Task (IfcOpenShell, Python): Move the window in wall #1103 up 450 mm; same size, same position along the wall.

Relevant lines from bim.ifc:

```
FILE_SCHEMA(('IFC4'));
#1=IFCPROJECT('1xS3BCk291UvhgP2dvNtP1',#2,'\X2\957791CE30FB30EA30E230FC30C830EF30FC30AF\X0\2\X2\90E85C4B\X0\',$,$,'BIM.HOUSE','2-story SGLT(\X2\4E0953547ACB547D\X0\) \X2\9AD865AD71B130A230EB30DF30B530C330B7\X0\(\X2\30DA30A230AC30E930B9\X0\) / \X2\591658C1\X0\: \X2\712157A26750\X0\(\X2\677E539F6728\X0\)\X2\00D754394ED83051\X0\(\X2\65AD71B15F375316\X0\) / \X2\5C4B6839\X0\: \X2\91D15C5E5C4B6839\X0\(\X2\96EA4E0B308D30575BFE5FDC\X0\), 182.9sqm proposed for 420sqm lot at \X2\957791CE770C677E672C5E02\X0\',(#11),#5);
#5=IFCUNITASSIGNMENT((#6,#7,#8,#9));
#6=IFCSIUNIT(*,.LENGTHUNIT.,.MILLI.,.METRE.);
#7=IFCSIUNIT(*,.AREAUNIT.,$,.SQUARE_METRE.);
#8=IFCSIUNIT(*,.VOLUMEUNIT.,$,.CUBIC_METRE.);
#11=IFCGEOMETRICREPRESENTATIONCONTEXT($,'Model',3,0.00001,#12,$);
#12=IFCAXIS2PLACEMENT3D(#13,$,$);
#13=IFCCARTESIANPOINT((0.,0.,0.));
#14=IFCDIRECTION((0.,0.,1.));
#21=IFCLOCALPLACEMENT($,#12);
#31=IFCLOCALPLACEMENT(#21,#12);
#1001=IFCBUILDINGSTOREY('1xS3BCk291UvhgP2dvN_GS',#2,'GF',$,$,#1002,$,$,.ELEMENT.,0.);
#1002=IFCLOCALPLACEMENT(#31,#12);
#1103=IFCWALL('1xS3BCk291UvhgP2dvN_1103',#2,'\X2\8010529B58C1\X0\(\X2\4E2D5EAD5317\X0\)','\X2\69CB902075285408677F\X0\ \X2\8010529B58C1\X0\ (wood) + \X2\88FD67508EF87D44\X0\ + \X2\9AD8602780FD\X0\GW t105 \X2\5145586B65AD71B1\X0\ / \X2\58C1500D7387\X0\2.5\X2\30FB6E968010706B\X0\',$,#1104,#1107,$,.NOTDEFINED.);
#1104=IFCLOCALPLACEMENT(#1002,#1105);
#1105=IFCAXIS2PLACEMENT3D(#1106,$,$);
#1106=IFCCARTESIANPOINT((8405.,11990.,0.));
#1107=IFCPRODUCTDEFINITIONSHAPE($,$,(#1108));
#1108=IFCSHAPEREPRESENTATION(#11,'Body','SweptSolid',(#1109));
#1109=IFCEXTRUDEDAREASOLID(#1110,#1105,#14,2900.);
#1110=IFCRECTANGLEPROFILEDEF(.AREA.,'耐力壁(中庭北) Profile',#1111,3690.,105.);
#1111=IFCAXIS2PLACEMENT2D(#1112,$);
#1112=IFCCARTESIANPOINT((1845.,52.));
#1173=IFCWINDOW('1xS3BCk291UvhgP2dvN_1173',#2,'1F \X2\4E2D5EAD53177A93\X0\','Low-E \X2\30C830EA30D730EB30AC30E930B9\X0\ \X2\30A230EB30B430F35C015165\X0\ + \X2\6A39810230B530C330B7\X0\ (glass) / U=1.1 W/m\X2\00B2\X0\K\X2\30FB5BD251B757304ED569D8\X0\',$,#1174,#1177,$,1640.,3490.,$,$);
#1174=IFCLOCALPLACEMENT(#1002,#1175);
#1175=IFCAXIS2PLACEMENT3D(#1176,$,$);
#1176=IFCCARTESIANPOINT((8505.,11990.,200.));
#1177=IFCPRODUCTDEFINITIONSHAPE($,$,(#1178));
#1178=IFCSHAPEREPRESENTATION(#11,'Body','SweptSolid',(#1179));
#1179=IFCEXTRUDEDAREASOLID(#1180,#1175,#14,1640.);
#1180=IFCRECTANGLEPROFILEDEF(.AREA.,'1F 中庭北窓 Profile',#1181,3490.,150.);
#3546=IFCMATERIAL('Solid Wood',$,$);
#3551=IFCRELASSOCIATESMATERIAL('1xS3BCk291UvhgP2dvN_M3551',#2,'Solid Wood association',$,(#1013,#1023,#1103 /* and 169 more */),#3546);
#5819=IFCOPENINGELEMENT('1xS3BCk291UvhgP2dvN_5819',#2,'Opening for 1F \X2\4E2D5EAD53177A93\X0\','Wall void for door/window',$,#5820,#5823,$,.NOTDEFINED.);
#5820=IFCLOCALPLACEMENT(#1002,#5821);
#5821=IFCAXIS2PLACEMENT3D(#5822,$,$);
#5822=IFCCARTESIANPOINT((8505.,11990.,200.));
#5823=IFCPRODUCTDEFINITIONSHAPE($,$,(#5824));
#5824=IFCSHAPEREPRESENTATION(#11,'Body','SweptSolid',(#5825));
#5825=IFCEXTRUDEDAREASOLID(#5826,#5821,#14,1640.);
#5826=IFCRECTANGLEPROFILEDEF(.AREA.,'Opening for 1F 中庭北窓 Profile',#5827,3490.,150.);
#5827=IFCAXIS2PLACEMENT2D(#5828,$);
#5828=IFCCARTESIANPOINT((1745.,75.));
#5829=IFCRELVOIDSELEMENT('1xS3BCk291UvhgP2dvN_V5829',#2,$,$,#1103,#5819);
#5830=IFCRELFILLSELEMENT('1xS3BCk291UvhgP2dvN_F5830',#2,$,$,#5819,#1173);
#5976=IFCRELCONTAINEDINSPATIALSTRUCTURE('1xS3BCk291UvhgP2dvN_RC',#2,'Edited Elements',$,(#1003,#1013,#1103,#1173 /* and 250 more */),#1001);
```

```python
import numpy as np
import ifcopenshell
import ifcopenshell.api.geometry
import ifcopenshell.util.placement
import ifcopenshell.util.unit

model = ifcopenshell.open("bim.ifc")
unit_scale = ifcopenshell.util.unit.calculate_unit_scale(model)

window = model.by_guid("1xS3BCk291UvhgP2dvN_1173")
opening = window.FillsVoids[0].RelatingOpeningElement
dz = 450.0

shift = np.array([0.0, 0.0, dz])
# The window is not placed relative to its opening, so move both.
for product in (opening, window):
    matrix = ifcopenshell.util.placement.get_local_placement(product.ObjectPlacement)
    matrix[:3, 3] += shift
    ifcopenshell.api.geometry.edit_object_placement(model, product=product, matrix=matrix, is_si=False)

print(f"moved by {dz * unit_scale:+.3f} m")

model.write("bim-out.ifc")
```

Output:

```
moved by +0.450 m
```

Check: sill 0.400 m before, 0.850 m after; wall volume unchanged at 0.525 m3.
